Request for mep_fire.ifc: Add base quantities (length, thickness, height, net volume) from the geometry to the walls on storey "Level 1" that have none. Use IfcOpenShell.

First a look at what the model holds.

```python
import ifcopenshell
import ifcopenshell.util.element
import ifcopenshell.util.unit

model = ifcopenshell.open("mep_fire.ifc")
print(model.schema)
for unit_type in ("LENGTHUNIT", "AREAUNIT", "VOLUMEUNIT"):
    print(unit_type, ifcopenshell.util.unit.calculate_unit_scale(model, unit_type))
storey = next(s for s in model.by_type("IfcBuildingStorey") if s.Name == "Level 1")
walls = [e for e in ifcopenshell.util.element.get_decomposition(storey) if e.is_a("IfcWall")]
for e in sorted(walls, key=lambda e: e.id()):
    print(e.id(), e.is_a(), e.Name, list(ifcopenshell.util.element.get_psets(e, qtos_only=True)), sep=" | ")
```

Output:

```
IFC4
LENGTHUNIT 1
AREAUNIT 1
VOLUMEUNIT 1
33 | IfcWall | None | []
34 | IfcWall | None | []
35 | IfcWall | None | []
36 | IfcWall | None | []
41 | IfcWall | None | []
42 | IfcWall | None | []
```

```python
import ifcopenshell
import ifcopenshell.api.pset
import ifcopenshell.geom
import ifcopenshell.util.element
import ifcopenshell.util.shape
import ifcopenshell.util.unit

model = ifcopenshell.open("mep_fire.ifc")
unit_scale = ifcopenshell.util.unit.calculate_unit_scale(model)
volume_scale = ifcopenshell.util.unit.calculate_unit_scale(model, "VOLUMEUNIT")
settings = ifcopenshell.geom.settings()

storey = next(s for s in model.by_type("IfcBuildingStorey") if s.Name == "Level 1")
walls = [e for e in ifcopenshell.util.element.get_decomposition(storey) if e.is_a("IfcWall")]

for e in sorted(walls, key=lambda e: e.id()):
    if ifcopenshell.util.element.get_psets(e, qtos_only=True, should_inherit=False):
        continue
    # Geometry comes back in metres, in the element's own axes.
    shape = ifcopenshell.geom.create_shape(settings, e)
    values = {
        "Length": ifcopenshell.util.shape.get_x(shape.geometry) / unit_scale,
        "Width": ifcopenshell.util.shape.get_y(shape.geometry) / unit_scale,
        "Height": ifcopenshell.util.shape.get_z(shape.geometry) / unit_scale,
        "NetVolume": ifcopenshell.util.shape.get_volume(shape.geometry) / volume_scale,
    }
    qto = ifcopenshell.api.pset.add_qto(model, product=e, name="Qto_WallBaseQuantities")
    ifcopenshell.api.pset.edit_qto(model, qto=qto, properties=values)
    print(e.id(), {k: round(v, 3) for k, v in values.items()})

model.write("mep_fire_updated.ifc")
```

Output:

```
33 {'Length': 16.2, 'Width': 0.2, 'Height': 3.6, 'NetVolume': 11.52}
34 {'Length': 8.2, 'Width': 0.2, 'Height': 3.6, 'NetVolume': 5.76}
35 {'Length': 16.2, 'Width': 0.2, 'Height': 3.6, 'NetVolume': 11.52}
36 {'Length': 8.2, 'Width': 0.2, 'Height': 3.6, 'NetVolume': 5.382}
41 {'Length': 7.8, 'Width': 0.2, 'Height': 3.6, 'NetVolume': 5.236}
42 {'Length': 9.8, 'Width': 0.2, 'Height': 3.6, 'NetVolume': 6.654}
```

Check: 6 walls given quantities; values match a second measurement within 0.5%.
